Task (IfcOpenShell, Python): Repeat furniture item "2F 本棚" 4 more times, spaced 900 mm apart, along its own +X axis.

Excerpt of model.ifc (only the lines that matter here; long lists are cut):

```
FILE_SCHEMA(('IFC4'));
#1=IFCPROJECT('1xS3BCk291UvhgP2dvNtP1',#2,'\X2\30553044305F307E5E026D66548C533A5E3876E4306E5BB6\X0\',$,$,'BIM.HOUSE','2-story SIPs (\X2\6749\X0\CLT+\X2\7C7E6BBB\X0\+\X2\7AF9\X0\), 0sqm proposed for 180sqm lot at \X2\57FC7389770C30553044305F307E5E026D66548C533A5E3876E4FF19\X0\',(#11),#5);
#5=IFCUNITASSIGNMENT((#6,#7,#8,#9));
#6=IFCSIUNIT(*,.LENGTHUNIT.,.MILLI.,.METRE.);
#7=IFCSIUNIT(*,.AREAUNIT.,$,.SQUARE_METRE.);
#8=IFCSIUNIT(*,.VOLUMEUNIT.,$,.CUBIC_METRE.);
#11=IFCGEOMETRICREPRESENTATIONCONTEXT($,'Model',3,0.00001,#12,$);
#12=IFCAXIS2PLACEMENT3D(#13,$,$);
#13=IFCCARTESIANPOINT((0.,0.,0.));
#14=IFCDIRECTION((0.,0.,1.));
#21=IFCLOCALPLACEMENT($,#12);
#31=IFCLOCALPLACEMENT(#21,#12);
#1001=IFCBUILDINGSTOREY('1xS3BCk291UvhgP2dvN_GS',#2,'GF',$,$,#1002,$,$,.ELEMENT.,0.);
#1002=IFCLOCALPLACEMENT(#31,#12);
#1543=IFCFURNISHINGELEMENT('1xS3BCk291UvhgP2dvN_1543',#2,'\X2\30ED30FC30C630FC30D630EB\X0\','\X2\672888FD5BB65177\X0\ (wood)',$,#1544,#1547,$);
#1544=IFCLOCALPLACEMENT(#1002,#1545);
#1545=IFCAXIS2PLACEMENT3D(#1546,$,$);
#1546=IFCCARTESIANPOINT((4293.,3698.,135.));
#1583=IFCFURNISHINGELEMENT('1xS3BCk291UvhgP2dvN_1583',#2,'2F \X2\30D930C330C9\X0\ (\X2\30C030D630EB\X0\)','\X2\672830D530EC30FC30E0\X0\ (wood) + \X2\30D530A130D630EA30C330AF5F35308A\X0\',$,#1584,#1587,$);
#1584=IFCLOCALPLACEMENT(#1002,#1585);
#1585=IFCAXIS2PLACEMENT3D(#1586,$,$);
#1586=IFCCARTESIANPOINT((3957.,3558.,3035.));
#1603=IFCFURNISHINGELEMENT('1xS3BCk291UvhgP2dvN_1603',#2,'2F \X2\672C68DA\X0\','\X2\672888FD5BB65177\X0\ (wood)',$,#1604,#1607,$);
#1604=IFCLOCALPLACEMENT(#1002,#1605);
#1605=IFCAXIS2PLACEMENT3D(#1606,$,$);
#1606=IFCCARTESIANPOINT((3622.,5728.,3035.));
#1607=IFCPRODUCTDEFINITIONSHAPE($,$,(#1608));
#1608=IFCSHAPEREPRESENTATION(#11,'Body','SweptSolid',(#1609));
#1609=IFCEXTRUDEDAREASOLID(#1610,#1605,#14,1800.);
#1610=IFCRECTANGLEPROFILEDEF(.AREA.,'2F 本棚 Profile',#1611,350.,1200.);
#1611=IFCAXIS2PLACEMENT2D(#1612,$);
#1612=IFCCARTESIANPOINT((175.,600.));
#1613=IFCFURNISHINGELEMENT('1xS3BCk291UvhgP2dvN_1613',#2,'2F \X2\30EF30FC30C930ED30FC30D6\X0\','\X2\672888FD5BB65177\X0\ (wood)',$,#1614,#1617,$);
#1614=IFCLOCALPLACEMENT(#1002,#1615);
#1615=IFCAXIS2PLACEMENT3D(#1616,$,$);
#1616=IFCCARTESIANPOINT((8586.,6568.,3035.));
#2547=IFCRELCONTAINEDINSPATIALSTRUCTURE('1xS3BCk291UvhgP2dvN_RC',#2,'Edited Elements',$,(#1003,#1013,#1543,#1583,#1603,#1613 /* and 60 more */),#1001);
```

```python
import ifcopenshell
import ifcopenshell.api.geometry
import ifcopenshell.api.root
import ifcopenshell.util.element
import ifcopenshell.util.placement

model = ifcopenshell.open("model.ifc")


def reuse_history(source, copy):
    """copy_class also copies each property set's owner history, people and application; keep the originals."""
    for rel in copy.IsDefinedBy:
        if rel.is_a("IfcRelDefinesByProperties") and (history := rel.RelatingPropertyDefinition.OwnerHistory):
            rel.RelatingPropertyDefinition.OwnerHistory = source.OwnerHistory
            ifcopenshell.util.element.remove_deep2(model, history)


source = model.by_guid("1xS3BCk291UvhgP2dvN_1603")
base = ifcopenshell.util.placement.get_local_placement(source.ObjectPlacement)
step = base[:3, 0] * 900.0

for i in range(1, 5):
    copy = ifcopenshell.api.root.copy_class(model, product=source)
    copy.Representation = ifcopenshell.util.element.copy_deep(
        model, source.Representation, exclude=["IfcGeometricRepresentationContext", "IfcRepresentationMap"]
    )
    reuse_history(source, copy)
    matrix = base.copy()
    matrix[:3, 3] += i * step
    print("added at", matrix[:3, 3].round(3) + 0.0)
    ifcopenshell.api.geometry.edit_object_placement(model, product=copy, matrix=matrix, is_si=False)

model.write("model_rev.ifc")
```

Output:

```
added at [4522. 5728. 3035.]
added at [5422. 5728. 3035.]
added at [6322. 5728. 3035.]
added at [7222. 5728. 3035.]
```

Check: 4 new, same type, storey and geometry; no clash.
